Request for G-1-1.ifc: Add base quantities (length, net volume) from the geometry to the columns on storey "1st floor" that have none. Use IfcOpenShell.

First a look at what the model holds.

```python
import ifcopenshell
import ifcopenshell.util.element
import ifcopenshell.util.unit

model = ifcopenshell.open("G-1-1.ifc")
print(model.schema)
for unit_type in ("LENGTHUNIT", "AREAUNIT", "VOLUMEUNIT"):
    print(unit_type, ifcopenshell.util.unit.calculate_unit_scale(model, unit_type))
storey = next(s for s in model.by_type("IfcBuildingStorey") if s.Name == "1st floor")
columns = [e for e in ifcopenshell.util.element.get_decomposition(storey) if e.is_a("IfcColumn")]
for e in sorted(columns, key=lambda e: e.id()):
    print(e.id(), e.is_a(), e.Name, list(ifcopenshell.util.element.get_psets(e, qtos_only=True)), sep=" | ")
```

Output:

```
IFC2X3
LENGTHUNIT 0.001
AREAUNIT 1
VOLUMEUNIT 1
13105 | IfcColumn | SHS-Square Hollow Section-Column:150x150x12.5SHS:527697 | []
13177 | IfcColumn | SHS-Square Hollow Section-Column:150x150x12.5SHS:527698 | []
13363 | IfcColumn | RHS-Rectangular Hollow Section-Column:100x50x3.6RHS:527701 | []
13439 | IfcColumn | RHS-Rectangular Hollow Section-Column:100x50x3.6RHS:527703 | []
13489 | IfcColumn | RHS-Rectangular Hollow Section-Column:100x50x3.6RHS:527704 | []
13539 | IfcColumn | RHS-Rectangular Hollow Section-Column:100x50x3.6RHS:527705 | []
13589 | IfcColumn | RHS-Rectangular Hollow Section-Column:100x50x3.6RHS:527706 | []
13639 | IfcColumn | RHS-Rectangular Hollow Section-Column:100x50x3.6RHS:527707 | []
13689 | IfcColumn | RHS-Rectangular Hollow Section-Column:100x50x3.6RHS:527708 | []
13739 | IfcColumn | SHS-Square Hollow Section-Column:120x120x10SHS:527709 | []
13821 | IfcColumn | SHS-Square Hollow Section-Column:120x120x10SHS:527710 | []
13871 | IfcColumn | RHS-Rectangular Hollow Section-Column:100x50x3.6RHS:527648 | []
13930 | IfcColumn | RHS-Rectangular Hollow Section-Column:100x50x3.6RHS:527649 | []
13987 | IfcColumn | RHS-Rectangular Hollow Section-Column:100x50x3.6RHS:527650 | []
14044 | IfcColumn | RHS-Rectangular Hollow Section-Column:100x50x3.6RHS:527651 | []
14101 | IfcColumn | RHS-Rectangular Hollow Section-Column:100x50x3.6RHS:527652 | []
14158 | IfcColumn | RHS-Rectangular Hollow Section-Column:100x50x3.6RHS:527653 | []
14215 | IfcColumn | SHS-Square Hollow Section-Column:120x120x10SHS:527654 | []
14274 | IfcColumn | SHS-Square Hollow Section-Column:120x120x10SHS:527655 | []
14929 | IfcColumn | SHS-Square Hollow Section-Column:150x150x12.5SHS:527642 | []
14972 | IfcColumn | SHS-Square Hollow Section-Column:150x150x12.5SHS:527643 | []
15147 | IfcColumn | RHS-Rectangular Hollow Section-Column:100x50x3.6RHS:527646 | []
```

```python
import ifcopenshell
import ifcopenshell.api.pset
import ifcopenshell.geom
import ifcopenshell.util.element
import ifcopenshell.util.shape
import ifcopenshell.util.unit

model = ifcopenshell.open("G-1-1.ifc")
unit_scale = ifcopenshell.util.unit.calculate_unit_scale(model)
volume_scale = ifcopenshell.util.unit.calculate_unit_scale(model, "VOLUMEUNIT")
settings = ifcopenshell.geom.settings()

storey = next(s for s in model.by_type("IfcBuildingStorey") if s.Name == "1st floor")
columns = [e for e in ifcopenshell.util.element.get_decomposition(storey) if e.is_a("IfcColumn")]

for e in sorted(columns, key=lambda e: e.id()):
    if ifcopenshell.util.element.get_psets(e, qtos_only=True, should_inherit=False):
        continue
    # Geometry comes back in metres, in the element's own axes.
    shape = ifcopenshell.geom.create_shape(settings, e)
    values = {
        "Length": ifcopenshell.util.shape.get_z(shape.geometry) / unit_scale,
        "NetVolume": ifcopenshell.util.shape.get_volume(shape.geometry) / volume_scale,
    }
    qto = ifcopenshell.api.pset.add_qto(model, product=e, name="BaseQuantities")
    ifcopenshell.api.pset.edit_qto(model, qto=qto, properties=values)
    print(e.id(), {k: round(v, 3) for k, v in values.items()})

model.write("G-1-1-out.ifc")
```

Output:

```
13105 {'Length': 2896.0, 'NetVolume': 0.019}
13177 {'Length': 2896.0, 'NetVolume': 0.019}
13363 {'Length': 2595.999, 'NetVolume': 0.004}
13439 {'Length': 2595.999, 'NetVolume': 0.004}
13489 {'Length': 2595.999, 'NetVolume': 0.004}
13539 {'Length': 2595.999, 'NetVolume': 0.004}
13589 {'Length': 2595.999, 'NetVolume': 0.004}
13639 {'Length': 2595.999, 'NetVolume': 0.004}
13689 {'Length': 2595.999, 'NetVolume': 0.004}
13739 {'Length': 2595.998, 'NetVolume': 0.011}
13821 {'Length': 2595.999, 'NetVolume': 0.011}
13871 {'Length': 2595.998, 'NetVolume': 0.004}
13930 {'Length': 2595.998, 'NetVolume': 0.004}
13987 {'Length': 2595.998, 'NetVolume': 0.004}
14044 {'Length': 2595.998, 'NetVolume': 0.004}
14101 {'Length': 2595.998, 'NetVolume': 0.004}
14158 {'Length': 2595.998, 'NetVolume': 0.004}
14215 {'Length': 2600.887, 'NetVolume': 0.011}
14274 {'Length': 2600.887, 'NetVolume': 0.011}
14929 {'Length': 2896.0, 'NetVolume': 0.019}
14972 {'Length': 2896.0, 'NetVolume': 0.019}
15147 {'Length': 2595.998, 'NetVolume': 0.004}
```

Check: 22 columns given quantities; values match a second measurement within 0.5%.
